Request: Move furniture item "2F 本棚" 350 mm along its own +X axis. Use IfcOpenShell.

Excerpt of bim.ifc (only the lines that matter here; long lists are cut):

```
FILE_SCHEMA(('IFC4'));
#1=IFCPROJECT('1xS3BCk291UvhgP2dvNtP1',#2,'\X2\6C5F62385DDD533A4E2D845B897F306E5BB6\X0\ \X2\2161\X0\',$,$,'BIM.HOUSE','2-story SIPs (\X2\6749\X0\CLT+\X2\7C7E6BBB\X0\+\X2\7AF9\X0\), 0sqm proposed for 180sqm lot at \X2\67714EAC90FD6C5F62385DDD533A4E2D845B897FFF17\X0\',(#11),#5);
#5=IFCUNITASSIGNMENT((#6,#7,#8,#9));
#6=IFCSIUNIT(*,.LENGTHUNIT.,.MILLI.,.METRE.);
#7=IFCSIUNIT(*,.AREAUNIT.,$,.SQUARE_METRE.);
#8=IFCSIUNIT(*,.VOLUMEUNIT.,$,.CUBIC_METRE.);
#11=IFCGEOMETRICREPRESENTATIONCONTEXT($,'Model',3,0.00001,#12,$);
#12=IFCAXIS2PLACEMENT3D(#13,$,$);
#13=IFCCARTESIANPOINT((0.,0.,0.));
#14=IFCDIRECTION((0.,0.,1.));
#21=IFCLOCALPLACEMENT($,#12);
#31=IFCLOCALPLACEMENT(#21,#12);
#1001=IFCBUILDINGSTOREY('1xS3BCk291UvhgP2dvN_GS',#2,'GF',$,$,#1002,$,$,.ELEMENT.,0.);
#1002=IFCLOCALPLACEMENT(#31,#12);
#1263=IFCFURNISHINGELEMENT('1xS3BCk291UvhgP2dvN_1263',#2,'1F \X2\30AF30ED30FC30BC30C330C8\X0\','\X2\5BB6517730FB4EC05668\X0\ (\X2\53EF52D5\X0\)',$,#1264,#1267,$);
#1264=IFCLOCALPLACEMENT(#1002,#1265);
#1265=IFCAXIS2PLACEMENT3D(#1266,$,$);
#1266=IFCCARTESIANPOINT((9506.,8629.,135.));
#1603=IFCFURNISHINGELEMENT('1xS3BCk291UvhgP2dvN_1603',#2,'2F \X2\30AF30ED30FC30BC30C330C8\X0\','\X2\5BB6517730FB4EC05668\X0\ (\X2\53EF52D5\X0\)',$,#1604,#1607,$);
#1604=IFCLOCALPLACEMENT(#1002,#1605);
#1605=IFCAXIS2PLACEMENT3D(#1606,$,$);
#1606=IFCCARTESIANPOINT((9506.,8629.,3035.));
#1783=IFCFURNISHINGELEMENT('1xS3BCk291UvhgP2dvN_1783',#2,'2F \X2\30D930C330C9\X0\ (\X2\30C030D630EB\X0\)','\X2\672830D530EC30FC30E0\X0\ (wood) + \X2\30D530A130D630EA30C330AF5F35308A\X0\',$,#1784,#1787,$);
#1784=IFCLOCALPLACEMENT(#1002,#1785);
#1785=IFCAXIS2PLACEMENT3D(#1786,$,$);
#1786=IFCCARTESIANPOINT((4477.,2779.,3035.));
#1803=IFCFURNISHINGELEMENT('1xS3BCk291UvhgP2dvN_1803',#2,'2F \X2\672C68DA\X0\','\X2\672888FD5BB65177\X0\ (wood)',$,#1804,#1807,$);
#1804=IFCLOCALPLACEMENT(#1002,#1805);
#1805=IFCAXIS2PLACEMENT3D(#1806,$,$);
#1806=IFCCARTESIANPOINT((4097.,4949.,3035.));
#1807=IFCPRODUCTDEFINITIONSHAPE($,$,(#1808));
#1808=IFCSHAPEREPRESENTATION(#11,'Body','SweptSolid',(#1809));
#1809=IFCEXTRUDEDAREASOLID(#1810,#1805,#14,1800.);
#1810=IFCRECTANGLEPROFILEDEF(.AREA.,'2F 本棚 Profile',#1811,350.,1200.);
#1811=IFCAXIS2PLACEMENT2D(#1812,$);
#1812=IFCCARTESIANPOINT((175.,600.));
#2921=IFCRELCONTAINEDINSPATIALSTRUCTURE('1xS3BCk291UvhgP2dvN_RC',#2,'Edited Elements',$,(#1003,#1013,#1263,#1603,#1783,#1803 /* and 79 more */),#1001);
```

```python
import ifcopenshell
import ifcopenshell.api.geometry
import ifcopenshell.util.placement

model = ifcopenshell.open("bim.ifc")

item = model.by_guid("1xS3BCk291UvhgP2dvN_1803")
matrix = ifcopenshell.util.placement.get_local_placement(item.ObjectPlacement)
matrix[:3, 3] += matrix[:3, 0] * 350.0
ifcopenshell.api.geometry.edit_object_placement(model, product=item, matrix=matrix, is_si=False)

print(ifcopenshell.util.placement.get_local_placement(item.ObjectPlacement).round(3) + 0.0)

model.write("bim_updated.ifc")
```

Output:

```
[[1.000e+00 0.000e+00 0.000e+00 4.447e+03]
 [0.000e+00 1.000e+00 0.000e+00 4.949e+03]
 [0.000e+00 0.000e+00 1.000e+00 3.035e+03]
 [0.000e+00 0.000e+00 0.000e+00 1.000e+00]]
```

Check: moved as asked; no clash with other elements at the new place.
